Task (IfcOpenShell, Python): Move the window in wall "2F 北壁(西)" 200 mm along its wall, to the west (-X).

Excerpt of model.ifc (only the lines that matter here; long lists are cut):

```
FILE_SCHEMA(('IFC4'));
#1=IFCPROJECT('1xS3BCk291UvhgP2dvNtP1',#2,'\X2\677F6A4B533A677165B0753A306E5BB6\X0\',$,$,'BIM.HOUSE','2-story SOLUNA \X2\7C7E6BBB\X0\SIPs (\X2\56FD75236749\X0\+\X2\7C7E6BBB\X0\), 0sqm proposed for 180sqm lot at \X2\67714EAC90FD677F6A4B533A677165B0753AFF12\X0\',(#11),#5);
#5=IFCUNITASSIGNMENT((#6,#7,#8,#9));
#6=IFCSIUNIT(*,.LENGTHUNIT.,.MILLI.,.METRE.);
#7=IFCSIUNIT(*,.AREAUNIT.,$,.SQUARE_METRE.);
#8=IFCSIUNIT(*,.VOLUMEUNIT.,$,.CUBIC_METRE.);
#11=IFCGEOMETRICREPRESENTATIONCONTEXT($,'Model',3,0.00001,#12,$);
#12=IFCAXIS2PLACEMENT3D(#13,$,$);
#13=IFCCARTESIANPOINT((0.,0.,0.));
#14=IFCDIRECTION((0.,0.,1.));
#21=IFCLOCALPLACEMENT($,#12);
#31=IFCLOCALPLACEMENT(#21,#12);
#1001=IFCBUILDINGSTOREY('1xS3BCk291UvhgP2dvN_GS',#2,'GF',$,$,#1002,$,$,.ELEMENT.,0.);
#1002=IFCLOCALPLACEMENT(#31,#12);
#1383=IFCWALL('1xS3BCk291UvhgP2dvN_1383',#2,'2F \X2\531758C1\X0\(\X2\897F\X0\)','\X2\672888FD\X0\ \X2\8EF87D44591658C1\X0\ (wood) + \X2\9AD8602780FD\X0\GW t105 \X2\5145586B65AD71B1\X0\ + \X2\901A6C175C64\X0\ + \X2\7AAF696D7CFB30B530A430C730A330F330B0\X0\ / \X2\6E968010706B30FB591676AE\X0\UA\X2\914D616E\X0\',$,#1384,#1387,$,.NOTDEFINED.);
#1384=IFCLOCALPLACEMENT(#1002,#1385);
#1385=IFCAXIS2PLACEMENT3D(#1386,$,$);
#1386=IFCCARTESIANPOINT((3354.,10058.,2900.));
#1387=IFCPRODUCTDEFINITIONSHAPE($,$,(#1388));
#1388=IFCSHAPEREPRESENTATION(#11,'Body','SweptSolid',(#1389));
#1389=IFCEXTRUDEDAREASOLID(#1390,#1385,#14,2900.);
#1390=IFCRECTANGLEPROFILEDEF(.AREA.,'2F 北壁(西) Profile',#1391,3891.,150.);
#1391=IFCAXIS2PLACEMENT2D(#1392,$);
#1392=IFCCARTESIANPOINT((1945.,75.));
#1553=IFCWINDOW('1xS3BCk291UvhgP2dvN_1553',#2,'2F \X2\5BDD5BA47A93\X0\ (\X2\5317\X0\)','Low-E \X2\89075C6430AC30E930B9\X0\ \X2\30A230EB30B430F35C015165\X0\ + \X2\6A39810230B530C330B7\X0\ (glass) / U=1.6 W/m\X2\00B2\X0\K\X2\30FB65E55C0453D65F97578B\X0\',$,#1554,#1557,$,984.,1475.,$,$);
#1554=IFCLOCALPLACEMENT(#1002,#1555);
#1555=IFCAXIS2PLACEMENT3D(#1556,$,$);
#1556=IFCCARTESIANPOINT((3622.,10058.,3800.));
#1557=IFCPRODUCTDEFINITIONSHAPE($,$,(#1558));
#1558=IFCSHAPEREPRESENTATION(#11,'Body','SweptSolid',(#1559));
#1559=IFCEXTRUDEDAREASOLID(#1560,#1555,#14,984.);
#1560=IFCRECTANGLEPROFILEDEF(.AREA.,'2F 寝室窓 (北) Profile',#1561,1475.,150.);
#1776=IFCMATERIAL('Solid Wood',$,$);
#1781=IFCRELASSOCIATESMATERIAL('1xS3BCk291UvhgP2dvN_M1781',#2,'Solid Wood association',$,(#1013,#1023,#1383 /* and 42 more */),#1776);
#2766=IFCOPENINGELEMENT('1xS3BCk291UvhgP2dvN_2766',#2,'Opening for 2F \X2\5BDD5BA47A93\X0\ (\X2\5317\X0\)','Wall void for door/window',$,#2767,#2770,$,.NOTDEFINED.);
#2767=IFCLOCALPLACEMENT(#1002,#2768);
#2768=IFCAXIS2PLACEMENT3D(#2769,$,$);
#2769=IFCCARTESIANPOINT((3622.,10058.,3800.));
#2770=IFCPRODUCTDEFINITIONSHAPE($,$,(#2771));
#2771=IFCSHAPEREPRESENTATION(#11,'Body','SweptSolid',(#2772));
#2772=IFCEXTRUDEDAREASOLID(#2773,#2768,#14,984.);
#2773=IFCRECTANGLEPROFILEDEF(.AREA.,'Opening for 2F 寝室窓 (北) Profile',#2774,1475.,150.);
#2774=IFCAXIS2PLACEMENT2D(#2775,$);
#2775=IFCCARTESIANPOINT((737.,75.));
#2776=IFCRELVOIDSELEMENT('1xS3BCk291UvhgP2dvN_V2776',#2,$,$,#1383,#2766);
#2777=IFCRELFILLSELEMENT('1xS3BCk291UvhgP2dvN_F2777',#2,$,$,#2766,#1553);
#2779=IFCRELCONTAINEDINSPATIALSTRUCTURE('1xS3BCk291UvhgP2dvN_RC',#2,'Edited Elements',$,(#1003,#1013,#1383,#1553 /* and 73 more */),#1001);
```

```python
import ifcopenshell
import ifcopenshell.api.geometry
import ifcopenshell.util.placement

model = ifcopenshell.open("model.ifc")

window = model.by_guid("1xS3BCk291UvhgP2dvN_1553")
opening = window.FillsVoids[0].RelatingOpeningElement
wall = opening.VoidsElements[0].RelatingBuildingElement

wall_matrix = ifcopenshell.util.placement.get_local_placement(wall.ObjectPlacement)
shift = wall_matrix[:3, 0] * -200.0
before = ifcopenshell.util.placement.get_local_placement(window.ObjectPlacement)[:3, 3].copy()

# The window is not placed relative to its opening, so move both.
for product in (opening, window):
    matrix = ifcopenshell.util.placement.get_local_placement(product.ObjectPlacement)
    matrix[:3, 3] += shift
    ifcopenshell.api.geometry.edit_object_placement(model, product=product, matrix=matrix, is_si=False)

after = ifcopenshell.util.placement.get_local_placement(window.ObjectPlacement)[:3, 3]
print("window moved by", (after - before).round(3) + 0.0)

model.write("model_v2.ifc")
```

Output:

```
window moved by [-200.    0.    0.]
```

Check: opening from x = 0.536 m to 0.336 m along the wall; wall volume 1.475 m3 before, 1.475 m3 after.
